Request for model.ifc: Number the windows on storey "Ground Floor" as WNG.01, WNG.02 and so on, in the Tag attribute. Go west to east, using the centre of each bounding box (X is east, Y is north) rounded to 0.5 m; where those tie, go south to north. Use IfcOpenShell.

First a look at what the model holds.

```python
import ifcopenshell
import ifcopenshell.util.element
import ifcopenshell.util.placement

model = ifcopenshell.open("model.ifc")
print(model.schema)
storey = next(s for s in model.by_type("IfcBuildingStorey") if s.Name == "Ground Floor")
windows = [e for e in ifcopenshell.util.element.get_decomposition(storey) if e.is_a("IfcWindow")]
for e in sorted(windows, key=lambda e: e.id()):
    origin = ifcopenshell.util.placement.get_local_placement(e.ObjectPlacement)[:3, 3]
    print(e.id(), e.Tag, e.Name, origin.round(2) + 0.0, sep=" | ")
```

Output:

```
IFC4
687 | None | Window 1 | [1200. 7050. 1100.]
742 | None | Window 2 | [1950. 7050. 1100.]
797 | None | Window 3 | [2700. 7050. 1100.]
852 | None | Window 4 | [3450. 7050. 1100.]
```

```python
import ifcopenshell
import ifcopenshell.geom
import ifcopenshell.util.element
import ifcopenshell.util.shape

model = ifcopenshell.open("model.ifc")
settings = ifcopenshell.geom.settings()
settings.set("use-world-coords", True)


def centre(element):
    shape = ifcopenshell.geom.create_shape(settings, element)
    return ifcopenshell.util.shape.get_bbox_centroid(shape.geometry)


storey = next(s for s in model.by_type("IfcBuildingStorey") if s.Name == "Ground Floor")
windows = [e for e in ifcopenshell.util.element.get_decomposition(storey) if e.is_a("IfcWindow")]

# Insertion points can sit at a corner or the storey origin, so sort by the geometry (in metres).
centres = {e: centre(e) for e in windows}
windows.sort(key=lambda e: (round(centres[e][0] / 0.5), centres[e][1]))

for i, e in enumerate(windows, start=1):
    number = f"WNG.{i:02d}"
    e.Tag = number
    print(e.id(), number)

model.write("model_updated.ifc")
```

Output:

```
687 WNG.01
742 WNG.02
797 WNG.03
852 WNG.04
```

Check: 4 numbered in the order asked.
